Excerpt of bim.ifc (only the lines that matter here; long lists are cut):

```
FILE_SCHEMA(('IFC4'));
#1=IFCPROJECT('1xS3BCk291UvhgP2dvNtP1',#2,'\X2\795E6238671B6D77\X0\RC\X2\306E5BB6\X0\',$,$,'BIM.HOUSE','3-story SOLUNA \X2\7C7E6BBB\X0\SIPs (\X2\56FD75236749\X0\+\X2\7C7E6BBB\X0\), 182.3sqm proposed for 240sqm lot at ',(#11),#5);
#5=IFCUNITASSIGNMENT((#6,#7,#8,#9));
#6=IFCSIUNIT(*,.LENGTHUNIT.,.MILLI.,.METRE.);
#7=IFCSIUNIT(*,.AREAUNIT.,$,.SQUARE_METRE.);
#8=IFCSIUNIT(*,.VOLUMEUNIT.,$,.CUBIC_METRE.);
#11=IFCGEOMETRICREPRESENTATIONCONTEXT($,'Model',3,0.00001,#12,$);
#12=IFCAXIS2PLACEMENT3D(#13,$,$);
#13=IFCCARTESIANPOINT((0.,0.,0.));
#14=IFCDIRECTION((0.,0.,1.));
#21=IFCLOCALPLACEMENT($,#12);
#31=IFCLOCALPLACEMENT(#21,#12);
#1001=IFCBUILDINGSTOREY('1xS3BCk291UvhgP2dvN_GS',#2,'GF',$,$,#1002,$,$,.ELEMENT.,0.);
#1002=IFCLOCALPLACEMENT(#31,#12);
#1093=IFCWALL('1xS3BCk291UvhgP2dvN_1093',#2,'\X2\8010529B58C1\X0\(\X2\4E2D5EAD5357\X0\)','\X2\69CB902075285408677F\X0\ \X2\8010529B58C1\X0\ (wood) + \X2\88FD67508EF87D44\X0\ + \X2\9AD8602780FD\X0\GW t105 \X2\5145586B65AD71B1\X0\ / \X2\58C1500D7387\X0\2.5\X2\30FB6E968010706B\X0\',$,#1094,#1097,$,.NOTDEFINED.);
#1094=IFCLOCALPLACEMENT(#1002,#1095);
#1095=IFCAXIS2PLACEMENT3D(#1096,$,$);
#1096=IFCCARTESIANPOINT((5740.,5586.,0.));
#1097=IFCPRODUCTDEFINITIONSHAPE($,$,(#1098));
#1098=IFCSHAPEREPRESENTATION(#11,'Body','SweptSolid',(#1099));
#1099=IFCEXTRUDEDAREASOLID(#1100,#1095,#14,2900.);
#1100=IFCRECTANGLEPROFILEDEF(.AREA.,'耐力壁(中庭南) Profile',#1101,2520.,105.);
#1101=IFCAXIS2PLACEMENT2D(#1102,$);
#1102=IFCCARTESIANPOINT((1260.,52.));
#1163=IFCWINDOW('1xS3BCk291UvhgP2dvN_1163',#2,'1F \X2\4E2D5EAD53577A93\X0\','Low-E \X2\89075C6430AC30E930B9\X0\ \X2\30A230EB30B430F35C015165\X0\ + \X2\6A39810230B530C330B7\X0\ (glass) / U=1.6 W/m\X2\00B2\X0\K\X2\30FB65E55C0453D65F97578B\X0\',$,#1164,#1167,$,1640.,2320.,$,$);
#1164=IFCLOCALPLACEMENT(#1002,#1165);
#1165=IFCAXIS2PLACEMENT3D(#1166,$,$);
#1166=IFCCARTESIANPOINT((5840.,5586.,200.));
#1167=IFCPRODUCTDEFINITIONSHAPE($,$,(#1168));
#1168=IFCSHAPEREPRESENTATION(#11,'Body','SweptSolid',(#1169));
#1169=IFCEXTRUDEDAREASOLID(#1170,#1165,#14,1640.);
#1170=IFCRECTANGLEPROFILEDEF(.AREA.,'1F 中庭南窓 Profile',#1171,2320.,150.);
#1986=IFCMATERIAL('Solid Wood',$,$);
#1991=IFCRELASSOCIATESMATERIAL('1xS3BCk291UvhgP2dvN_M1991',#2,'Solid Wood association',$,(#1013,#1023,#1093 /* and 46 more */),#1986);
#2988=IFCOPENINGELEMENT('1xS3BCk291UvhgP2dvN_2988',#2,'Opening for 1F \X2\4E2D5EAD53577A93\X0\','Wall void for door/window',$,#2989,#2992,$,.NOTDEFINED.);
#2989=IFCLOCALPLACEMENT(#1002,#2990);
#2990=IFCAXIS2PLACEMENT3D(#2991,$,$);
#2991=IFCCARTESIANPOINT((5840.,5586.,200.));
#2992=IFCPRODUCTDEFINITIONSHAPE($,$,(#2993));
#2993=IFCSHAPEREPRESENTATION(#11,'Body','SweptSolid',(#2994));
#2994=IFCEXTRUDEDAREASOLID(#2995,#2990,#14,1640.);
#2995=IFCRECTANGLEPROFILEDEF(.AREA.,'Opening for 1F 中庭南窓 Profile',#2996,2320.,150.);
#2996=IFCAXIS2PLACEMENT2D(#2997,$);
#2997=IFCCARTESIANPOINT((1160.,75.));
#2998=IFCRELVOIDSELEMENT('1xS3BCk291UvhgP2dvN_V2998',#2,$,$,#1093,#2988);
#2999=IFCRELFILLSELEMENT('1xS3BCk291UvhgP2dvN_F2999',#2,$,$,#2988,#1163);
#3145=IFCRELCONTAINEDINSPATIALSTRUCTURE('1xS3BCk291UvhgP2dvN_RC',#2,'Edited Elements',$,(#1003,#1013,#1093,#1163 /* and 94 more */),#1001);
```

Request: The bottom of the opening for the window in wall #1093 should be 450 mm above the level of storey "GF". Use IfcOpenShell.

```python
import numpy as np
import ifcopenshell
import ifcopenshell.api.geometry
import ifcopenshell.geom
import ifcopenshell.util.element
import ifcopenshell.util.placement
import ifcopenshell.util.shape
import ifcopenshell.util.unit

model = ifcopenshell.open("bim.ifc")
unit_scale = ifcopenshell.util.unit.calculate_unit_scale(model)

window = model.by_guid("1xS3BCk291UvhgP2dvN_1163")
opening = window.FillsVoids[0].RelatingOpeningElement
storey = ifcopenshell.util.element.get_container(window, ifc_class="IfcBuildingStorey")
level = ifcopenshell.util.placement.get_local_placement(storey.ObjectPlacement)[2, 3]

# The opening's origin need not be at the sill, so measure its lowest point.
shape = ifcopenshell.geom.create_shape(ifcopenshell.geom.settings(), opening)
bottom = ifcopenshell.util.shape.get_shape_bottom_elevation(shape, shape.geometry) / unit_scale
dz = level + 0.45 / unit_scale - bottom

shift = np.array([0.0, 0.0, dz])
# The window is not placed relative to its opening, so move both.
for product in (opening, window):
    matrix = ifcopenshell.util.placement.get_local_placement(product.ObjectPlacement)
    matrix[:3, 3] += shift
    ifcopenshell.api.geometry.edit_object_placement(model, product=product, matrix=matrix, is_si=False)

print(f"moved by {dz * unit_scale:+.3f} m")

model.write("bim_edited.ifc")
```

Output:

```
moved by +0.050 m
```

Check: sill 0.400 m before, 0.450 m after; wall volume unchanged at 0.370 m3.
